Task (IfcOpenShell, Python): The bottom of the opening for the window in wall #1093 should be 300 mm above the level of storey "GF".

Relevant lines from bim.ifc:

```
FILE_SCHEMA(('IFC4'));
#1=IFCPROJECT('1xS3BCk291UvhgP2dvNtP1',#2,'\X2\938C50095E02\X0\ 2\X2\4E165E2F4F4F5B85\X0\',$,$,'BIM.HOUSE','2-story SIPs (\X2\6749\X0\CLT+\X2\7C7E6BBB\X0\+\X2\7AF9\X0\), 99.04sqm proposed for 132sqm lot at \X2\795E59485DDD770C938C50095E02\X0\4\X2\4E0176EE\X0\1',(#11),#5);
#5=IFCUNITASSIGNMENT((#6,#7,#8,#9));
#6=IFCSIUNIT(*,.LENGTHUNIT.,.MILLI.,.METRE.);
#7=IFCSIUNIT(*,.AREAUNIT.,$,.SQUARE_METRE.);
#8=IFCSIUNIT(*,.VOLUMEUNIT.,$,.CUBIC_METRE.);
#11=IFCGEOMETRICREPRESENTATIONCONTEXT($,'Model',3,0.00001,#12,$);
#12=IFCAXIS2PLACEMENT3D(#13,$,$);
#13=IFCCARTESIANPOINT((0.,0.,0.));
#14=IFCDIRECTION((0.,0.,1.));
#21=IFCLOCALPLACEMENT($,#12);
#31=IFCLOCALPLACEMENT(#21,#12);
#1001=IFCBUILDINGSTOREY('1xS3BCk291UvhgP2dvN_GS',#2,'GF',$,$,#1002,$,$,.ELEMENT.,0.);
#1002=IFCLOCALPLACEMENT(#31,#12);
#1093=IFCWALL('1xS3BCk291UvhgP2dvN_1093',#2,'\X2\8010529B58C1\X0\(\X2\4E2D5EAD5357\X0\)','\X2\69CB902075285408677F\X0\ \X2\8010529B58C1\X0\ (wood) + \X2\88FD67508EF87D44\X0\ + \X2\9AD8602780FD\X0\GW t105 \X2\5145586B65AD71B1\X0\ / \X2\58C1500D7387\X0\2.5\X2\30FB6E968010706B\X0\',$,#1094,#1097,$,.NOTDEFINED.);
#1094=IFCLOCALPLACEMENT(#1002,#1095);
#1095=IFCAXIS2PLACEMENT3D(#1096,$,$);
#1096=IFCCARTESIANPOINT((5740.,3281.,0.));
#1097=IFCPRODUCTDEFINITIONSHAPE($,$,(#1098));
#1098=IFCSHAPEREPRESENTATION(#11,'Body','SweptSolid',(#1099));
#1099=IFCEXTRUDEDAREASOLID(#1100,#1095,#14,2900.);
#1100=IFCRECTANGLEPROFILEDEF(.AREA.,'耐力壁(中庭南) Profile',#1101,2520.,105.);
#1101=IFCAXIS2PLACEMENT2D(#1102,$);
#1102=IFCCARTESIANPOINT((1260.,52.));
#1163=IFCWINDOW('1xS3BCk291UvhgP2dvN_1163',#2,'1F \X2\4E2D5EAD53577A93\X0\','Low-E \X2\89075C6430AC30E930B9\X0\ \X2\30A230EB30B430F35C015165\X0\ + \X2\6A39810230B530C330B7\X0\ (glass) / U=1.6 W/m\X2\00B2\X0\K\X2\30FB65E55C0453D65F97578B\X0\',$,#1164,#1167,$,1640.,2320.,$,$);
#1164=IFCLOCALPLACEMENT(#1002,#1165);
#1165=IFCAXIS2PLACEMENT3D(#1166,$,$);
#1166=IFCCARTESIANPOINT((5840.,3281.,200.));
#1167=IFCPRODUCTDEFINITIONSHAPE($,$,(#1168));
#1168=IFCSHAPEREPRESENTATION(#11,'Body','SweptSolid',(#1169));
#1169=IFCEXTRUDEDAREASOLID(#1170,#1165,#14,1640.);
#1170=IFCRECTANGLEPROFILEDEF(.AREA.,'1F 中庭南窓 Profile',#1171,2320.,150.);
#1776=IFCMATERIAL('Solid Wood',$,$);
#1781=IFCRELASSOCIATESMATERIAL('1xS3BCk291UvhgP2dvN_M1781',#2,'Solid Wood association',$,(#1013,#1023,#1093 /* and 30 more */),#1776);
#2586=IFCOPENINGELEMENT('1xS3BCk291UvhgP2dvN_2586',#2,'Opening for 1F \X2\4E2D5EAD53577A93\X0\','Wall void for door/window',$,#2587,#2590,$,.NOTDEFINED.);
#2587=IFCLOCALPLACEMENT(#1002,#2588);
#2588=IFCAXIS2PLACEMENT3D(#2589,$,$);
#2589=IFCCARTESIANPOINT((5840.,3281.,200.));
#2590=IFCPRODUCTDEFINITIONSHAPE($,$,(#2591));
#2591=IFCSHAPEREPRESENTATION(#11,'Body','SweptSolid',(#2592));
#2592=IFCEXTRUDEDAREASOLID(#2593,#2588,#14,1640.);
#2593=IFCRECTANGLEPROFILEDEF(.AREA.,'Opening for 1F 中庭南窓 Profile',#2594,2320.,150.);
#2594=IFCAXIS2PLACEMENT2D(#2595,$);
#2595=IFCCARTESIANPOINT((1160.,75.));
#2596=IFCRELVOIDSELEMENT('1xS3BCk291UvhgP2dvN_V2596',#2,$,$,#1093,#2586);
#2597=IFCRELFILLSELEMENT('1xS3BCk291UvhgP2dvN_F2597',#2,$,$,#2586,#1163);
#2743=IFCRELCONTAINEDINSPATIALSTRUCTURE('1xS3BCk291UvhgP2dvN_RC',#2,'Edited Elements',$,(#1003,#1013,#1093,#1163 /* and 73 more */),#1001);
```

```python
import numpy as np
import ifcopenshell
import ifcopenshell.api.geometry
import ifcopenshell.geom
import ifcopenshell.util.element
import ifcopenshell.util.placement
import ifcopenshell.util.shape
import ifcopenshell.util.unit

model = ifcopenshell.open("bim.ifc")
unit_scale = ifcopenshell.util.unit.calculate_unit_scale(model)

window = model.by_guid("1xS3BCk291UvhgP2dvN_1163")
opening = window.FillsVoids[0].RelatingOpeningElement
storey = ifcopenshell.util.element.get_container(window, ifc_class="IfcBuildingStorey")
level = ifcopenshell.util.placement.get_local_placement(storey.ObjectPlacement)[2, 3]

# The opening's origin need not be at the sill, so measure its lowest point.
shape = ifcopenshell.geom.create_shape(ifcopenshell.geom.settings(), opening)
bottom = ifcopenshell.util.shape.get_shape_bottom_elevation(shape, shape.geometry) / unit_scale
dz = level + 0.3 / unit_scale - bottom

shift = np.array([0.0, 0.0, dz])
# The window is not placed relative to its opening, so move both.
for product in (opening, window):
    matrix = ifcopenshell.util.placement.get_local_placement(product.ObjectPlacement)
    matrix[:3, 3] += shift
    ifcopenshell.api.geometry.edit_object_placement(model, product=product, matrix=matrix, is_si=False)

print(f"moved by {dz * unit_scale:+.3f} m")

model.write("bim_v2.ifc")
```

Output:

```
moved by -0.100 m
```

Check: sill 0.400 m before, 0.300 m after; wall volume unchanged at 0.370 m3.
